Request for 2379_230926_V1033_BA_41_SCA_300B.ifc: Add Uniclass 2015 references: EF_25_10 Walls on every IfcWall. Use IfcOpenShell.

First a look at what the model holds.

```python
import ifcopenshell

model = ifcopenshell.open("2379_230926_V1033_BA_41_SCA_300B.ifc")
print(model.schema)
print("classifications:", [c.Name for c in model.by_type("IfcClassification")])
for ifc_class in ("IfcDoor", "IfcRoof", "IfcStair", "IfcWall", "IfcWindow"):
    print(ifc_class, len(model.by_type(ifc_class)))
```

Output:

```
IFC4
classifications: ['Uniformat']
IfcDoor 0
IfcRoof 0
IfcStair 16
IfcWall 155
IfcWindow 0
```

```python
import ifcopenshell
import ifcopenshell.api.classification

model = ifcopenshell.open("2379_230926_V1033_BA_41_SCA_300B.ifc")

system = ifcopenshell.api.classification.add_classification(model, classification="Uniclass 2015")

codes = {
    "IfcWall": ("EF_25_10", "Walls"),
}
for ifc_class, (code, name) in codes.items():
    products = model.by_type(ifc_class)
    ifcopenshell.api.classification.add_reference(
        model, products=products, classification=system, identification=code, name=name
    )
    print(code, len(products))

model.write("2379_230926_V1033_BA_41_SCA_300B_edited.ifc")
```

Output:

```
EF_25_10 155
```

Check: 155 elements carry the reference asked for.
